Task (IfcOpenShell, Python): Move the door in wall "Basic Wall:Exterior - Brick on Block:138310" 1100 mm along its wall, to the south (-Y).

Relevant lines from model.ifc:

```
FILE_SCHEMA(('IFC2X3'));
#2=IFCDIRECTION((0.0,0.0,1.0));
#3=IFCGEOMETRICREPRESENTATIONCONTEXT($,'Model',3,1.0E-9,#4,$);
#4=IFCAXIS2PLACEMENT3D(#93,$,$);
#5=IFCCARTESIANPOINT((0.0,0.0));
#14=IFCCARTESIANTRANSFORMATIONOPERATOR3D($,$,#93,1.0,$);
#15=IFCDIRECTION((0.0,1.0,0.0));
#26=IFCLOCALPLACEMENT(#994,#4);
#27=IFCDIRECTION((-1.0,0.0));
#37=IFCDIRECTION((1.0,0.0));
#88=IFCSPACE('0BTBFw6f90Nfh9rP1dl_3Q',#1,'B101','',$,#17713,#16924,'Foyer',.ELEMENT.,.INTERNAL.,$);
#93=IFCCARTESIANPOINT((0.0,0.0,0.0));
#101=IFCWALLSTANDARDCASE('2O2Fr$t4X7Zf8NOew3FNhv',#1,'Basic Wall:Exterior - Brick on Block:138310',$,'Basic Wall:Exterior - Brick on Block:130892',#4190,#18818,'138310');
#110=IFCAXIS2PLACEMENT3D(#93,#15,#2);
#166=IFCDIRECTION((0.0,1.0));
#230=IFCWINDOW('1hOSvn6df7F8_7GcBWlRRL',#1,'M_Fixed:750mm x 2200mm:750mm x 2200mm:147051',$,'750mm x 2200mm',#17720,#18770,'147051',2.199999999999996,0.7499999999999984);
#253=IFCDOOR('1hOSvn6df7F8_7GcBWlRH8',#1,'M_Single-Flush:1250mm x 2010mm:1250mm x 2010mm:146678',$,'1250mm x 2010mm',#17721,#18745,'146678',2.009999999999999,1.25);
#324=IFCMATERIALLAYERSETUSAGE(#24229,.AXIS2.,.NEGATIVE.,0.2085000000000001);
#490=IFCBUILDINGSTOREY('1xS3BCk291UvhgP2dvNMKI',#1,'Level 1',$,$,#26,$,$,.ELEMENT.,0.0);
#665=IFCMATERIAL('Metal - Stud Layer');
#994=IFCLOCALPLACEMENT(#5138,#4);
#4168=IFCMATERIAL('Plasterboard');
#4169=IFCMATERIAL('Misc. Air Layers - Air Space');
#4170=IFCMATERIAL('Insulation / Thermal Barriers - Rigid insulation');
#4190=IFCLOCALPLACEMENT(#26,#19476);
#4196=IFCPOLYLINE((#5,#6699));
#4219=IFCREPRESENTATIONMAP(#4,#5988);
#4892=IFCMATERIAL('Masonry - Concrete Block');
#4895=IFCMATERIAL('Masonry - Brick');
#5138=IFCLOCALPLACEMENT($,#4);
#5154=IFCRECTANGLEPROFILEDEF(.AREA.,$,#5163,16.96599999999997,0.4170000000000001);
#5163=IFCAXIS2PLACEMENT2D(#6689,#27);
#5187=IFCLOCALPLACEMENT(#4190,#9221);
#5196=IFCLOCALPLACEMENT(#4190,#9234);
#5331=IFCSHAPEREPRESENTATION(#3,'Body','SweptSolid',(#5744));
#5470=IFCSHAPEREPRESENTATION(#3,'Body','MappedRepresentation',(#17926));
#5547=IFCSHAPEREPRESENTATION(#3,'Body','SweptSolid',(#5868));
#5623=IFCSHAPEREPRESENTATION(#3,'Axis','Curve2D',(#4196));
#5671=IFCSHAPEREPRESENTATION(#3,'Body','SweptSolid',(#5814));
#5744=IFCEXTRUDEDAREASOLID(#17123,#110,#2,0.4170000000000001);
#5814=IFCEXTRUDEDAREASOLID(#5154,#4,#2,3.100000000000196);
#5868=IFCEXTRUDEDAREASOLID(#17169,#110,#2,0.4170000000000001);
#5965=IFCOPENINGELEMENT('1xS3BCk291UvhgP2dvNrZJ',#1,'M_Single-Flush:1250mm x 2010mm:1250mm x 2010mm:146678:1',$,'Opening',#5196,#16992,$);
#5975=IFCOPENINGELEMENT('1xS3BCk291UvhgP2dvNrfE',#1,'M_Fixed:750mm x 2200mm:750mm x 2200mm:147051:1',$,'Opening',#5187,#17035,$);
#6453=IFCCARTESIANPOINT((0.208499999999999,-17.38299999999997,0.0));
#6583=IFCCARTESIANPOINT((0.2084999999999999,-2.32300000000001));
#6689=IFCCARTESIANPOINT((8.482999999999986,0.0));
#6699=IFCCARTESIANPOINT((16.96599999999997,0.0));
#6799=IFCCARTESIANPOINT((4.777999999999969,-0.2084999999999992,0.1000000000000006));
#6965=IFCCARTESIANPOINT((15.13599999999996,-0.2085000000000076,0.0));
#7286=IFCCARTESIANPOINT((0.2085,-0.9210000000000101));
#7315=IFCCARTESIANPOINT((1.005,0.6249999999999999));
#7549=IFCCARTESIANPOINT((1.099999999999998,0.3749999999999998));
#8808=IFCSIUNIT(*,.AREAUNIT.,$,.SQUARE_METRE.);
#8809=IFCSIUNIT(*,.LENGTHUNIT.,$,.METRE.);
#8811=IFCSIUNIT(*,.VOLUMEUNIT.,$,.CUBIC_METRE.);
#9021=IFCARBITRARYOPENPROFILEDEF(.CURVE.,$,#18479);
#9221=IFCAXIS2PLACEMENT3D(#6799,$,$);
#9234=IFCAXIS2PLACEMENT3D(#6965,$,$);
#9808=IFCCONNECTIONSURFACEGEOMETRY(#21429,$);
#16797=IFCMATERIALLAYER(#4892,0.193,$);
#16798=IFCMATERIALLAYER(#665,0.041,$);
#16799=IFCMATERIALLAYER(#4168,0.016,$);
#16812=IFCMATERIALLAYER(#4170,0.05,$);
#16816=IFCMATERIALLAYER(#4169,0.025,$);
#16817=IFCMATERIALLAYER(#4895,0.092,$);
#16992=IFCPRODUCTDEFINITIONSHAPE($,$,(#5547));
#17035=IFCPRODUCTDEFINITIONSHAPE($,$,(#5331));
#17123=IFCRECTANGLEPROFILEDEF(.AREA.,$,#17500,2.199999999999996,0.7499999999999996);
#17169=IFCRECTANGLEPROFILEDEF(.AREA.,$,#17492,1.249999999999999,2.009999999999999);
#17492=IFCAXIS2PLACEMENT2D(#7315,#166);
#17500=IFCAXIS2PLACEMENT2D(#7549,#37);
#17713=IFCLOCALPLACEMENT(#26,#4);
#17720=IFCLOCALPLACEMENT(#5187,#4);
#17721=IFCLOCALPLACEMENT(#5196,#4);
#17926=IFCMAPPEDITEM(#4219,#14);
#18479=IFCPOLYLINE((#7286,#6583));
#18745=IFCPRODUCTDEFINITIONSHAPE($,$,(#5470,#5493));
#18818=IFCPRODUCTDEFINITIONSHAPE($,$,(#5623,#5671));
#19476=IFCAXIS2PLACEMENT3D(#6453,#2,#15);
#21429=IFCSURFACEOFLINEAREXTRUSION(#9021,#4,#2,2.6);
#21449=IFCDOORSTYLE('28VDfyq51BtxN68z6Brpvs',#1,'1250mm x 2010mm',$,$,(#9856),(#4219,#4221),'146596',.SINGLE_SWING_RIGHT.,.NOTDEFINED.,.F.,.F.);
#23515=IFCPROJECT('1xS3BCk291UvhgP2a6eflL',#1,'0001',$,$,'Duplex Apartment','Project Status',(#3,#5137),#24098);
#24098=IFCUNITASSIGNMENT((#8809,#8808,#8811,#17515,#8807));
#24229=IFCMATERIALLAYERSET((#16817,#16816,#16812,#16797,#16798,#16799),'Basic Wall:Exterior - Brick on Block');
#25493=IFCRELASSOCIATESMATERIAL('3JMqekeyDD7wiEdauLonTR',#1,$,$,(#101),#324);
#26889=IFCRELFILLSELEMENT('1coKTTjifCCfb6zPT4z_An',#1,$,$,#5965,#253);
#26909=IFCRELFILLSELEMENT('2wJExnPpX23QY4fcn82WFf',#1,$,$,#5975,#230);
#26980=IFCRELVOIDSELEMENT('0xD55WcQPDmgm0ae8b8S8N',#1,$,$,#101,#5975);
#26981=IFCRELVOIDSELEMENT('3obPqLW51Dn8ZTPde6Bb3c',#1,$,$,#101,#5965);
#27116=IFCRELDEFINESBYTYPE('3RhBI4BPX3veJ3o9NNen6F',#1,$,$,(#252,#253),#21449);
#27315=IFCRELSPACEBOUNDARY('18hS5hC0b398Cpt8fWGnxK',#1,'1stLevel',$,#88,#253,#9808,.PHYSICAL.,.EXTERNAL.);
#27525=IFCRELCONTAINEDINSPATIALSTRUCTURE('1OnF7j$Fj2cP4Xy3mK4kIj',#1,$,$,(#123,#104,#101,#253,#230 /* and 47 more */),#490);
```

```python
import numpy as np
import ifcopenshell
import ifcopenshell.api.geometry
import ifcopenshell.util.placement
import ifcopenshell.util.unit

model = ifcopenshell.open("model.ifc")
unit_scale = ifcopenshell.util.unit.calculate_unit_scale(model)

door = model.by_guid("1hOSvn6df7F8_7GcBWlRH8")
opening = door.FillsVoids[0].RelatingOpeningElement
wall = opening.VoidsElements[0].RelatingBuildingElement

wall_matrix = ifcopenshell.util.placement.get_local_placement(wall.ObjectPlacement)
shift = wall_matrix[:3, 0] * -1.1 / unit_scale
before = ifcopenshell.util.placement.get_local_placement(door.ObjectPlacement)[:3, 3].copy()

# The door is placed relative to its opening, so it follows when the opening moves.
matrix = ifcopenshell.util.placement.get_local_placement(opening.ObjectPlacement)
matrix[:3, 3] += shift
ifcopenshell.api.geometry.edit_object_placement(
    model, product=opening, matrix=matrix, is_si=False, should_transform_children=True
)

# Space boundary surfaces are stored in each space's coordinates; move them too.
for rel in door.ProvidesBoundaries:
    if not rel.ConnectionGeometry:
        continue
    surface = rel.ConnectionGeometry.SurfaceOnRelatingElement
    space_matrix = ifcopenshell.util.placement.get_local_placement(rel.RelatingSpace.ObjectPlacement)
    point = np.array(surface.Position.Location.Coordinates) + space_matrix[:3, :3].T @ shift
    surface.Position = model.createIfcAxis2Placement3D(
        model.createIfcCartesianPoint(point.tolist()), surface.Position.Axis, surface.Position.RefDirection
    )

after = ifcopenshell.util.placement.get_local_placement(door.ObjectPlacement)[:3, 3]
print("door moved by", (after - before).round(3) + 0.0)

model.write("model-out.ifc")
```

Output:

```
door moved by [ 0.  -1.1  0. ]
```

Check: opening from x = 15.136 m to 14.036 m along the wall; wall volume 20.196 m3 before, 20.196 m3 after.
